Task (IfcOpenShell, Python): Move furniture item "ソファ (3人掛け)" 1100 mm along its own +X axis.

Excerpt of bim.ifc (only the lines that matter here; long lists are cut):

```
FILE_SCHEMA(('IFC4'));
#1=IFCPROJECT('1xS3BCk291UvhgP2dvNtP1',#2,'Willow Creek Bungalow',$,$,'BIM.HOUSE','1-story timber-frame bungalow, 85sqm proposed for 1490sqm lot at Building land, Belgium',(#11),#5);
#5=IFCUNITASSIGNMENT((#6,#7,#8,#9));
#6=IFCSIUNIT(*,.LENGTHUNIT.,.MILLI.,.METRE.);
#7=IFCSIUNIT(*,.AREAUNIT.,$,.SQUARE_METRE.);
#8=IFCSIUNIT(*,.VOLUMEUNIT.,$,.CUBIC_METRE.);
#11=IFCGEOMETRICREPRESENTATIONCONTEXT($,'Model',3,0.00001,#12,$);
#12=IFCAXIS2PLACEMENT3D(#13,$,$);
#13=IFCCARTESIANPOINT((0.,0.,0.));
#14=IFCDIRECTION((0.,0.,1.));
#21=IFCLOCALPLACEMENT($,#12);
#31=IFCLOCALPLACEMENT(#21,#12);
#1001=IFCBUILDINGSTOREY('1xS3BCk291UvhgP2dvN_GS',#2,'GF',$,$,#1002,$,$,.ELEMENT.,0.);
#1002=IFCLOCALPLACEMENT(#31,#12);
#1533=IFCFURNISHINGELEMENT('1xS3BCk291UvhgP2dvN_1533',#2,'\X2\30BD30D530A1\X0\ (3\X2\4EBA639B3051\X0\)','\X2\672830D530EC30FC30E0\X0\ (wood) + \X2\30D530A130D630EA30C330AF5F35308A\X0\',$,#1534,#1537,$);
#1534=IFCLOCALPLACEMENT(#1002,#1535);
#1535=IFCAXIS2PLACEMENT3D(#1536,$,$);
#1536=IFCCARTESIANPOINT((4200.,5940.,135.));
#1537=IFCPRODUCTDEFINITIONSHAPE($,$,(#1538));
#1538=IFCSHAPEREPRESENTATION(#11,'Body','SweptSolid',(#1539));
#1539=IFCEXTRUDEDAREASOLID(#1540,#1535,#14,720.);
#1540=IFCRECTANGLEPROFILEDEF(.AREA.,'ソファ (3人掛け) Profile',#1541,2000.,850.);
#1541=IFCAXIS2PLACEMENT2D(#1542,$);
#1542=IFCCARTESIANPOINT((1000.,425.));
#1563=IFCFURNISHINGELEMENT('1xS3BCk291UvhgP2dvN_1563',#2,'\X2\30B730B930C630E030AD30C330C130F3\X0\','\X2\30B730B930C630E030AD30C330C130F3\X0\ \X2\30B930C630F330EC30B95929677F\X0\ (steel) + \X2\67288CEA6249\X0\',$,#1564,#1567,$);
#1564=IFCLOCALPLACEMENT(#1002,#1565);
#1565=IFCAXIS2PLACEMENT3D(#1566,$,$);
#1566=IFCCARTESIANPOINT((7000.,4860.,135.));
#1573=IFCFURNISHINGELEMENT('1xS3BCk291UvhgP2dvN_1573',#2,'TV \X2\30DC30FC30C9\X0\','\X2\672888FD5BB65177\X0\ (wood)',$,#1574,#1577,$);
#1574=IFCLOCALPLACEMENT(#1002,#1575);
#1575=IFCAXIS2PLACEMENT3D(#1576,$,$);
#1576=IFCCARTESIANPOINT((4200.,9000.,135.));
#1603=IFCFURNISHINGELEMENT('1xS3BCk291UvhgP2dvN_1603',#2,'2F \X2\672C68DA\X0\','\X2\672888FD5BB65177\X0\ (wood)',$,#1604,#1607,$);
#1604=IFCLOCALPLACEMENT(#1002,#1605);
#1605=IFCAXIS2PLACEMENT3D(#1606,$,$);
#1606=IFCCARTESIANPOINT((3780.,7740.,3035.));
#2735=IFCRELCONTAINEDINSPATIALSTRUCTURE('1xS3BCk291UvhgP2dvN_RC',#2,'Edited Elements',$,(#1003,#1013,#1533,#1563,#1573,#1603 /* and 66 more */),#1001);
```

```python
import ifcopenshell
import ifcopenshell.api.geometry
import ifcopenshell.util.placement
import ifcopenshell.util.unit

model = ifcopenshell.open("bim.ifc")
unit_scale = ifcopenshell.util.unit.calculate_unit_scale(model)

item = model.by_guid("1xS3BCk291UvhgP2dvN_1533")
matrix = ifcopenshell.util.placement.get_local_placement(item.ObjectPlacement)
matrix[:3, 3] += matrix[:3, 0] * 1.1 / unit_scale
ifcopenshell.api.geometry.edit_object_placement(model, product=item, matrix=matrix, is_si=False)

print(ifcopenshell.util.placement.get_local_placement(item.ObjectPlacement).round(3) + 0.0)

model.write("bim_rev.ifc")
```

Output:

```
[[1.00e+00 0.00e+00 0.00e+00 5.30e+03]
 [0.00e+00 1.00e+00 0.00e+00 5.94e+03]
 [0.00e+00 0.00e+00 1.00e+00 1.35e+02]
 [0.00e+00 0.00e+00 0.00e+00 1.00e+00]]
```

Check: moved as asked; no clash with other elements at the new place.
